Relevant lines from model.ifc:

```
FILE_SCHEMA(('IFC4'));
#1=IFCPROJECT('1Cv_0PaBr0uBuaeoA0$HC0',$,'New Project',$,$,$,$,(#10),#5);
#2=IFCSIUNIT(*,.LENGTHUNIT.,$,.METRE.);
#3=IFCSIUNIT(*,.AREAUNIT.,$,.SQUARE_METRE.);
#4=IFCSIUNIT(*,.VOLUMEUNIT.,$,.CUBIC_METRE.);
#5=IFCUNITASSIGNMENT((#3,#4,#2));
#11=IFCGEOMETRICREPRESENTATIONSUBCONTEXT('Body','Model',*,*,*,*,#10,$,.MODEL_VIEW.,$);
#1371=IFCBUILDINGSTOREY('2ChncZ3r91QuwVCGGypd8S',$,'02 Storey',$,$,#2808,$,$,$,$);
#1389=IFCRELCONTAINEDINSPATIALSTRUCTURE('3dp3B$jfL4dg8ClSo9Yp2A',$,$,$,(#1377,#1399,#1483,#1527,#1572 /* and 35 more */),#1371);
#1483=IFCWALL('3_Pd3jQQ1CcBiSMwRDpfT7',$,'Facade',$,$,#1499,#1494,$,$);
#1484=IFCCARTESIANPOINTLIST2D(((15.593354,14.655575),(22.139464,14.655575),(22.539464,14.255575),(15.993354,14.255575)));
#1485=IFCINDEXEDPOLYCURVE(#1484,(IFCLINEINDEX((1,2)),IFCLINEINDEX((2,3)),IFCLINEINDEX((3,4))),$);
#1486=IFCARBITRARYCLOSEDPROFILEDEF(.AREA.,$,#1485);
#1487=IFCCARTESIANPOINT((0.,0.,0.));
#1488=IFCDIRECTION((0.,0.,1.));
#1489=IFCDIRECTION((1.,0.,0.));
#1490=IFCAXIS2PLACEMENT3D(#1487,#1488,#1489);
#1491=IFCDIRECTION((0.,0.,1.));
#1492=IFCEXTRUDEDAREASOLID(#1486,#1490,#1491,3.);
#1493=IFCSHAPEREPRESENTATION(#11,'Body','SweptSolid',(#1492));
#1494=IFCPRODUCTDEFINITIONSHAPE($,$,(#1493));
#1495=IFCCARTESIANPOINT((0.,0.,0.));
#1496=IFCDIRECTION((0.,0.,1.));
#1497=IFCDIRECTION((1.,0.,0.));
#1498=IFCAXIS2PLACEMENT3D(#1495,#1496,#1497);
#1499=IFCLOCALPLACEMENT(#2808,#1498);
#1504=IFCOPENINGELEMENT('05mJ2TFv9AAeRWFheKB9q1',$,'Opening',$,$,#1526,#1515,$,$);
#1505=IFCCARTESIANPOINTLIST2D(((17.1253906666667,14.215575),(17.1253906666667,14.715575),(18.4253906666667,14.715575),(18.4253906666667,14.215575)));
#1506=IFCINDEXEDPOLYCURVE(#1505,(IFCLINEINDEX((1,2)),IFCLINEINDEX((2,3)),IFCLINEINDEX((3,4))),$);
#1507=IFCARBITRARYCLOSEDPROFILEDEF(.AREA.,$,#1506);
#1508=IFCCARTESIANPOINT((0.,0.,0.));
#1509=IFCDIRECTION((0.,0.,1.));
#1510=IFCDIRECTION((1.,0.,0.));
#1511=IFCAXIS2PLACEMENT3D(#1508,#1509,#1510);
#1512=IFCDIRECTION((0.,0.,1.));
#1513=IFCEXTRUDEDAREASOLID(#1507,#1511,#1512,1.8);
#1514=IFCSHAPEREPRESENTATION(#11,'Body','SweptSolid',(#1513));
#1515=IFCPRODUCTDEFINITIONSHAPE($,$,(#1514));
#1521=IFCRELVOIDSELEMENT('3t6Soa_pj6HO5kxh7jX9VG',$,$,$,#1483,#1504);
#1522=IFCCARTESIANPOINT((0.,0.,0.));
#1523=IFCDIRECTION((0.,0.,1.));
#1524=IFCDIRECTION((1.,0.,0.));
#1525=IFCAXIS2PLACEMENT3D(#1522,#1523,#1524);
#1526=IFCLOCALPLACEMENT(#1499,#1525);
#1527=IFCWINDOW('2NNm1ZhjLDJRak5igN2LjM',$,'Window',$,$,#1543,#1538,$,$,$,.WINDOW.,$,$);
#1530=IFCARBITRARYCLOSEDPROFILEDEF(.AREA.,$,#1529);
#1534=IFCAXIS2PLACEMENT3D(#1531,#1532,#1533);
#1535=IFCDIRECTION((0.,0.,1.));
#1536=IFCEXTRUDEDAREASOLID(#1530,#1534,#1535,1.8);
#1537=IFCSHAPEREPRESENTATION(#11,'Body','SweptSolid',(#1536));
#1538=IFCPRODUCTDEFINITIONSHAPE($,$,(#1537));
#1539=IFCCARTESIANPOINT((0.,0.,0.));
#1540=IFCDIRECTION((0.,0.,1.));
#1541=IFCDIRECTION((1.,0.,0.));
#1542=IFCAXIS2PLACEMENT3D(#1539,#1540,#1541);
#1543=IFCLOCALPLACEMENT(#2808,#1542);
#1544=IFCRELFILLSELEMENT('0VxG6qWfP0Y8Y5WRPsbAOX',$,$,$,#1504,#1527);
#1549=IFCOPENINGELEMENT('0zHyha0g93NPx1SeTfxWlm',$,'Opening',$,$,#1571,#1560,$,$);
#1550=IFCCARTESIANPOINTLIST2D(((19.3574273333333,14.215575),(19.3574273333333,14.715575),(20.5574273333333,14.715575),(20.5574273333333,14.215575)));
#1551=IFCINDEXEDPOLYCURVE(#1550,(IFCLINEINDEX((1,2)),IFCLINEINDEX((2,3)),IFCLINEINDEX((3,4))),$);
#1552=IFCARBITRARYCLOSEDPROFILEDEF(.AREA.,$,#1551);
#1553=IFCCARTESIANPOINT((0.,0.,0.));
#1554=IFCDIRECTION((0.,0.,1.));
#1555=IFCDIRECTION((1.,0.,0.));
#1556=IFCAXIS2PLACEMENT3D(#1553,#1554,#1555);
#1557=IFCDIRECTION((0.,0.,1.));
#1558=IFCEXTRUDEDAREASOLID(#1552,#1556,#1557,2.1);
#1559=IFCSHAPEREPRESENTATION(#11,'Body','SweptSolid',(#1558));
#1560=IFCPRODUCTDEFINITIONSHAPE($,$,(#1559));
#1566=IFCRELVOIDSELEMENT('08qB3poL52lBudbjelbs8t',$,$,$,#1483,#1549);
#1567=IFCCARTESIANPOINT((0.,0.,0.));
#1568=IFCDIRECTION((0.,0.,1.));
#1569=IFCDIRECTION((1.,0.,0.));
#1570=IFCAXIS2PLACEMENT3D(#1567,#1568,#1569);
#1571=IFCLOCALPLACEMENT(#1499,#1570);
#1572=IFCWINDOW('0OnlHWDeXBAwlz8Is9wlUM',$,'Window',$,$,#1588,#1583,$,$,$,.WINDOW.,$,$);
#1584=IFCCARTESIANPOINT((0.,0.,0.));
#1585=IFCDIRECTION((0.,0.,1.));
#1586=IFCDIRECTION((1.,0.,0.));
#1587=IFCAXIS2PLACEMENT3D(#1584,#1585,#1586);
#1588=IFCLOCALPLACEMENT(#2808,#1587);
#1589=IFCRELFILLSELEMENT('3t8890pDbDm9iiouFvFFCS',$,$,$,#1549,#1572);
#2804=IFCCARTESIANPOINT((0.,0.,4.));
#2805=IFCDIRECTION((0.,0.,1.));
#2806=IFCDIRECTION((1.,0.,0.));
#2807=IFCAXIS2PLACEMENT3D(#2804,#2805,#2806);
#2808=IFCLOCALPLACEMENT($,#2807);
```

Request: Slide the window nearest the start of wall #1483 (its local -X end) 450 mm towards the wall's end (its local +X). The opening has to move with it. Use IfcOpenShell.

```python
import ifcopenshell
import ifcopenshell.api.geometry
import ifcopenshell.util.placement
import ifcopenshell.util.unit

model = ifcopenshell.open("model.ifc")
unit_scale = ifcopenshell.util.unit.calculate_unit_scale(model)

window = model.by_guid("2NNm1ZhjLDJRak5igN2LjM")
opening = window.FillsVoids[0].RelatingOpeningElement
wall = opening.VoidsElements[0].RelatingBuildingElement

wall_matrix = ifcopenshell.util.placement.get_local_placement(wall.ObjectPlacement)
shift = wall_matrix[:3, 0] * 0.45 / unit_scale
before = ifcopenshell.util.placement.get_local_placement(window.ObjectPlacement)[:3, 3].copy()

# The window is not placed relative to its opening, so move both.
for product in (opening, window):
    matrix = ifcopenshell.util.placement.get_local_placement(product.ObjectPlacement)
    matrix[:3, 3] += shift
    ifcopenshell.api.geometry.edit_object_placement(model, product=product, matrix=matrix, is_si=False)

after = ifcopenshell.util.placement.get_local_placement(window.ObjectPlacement)[:3, 3]
print("window moved by", (after - before).round(3) + 0.0)

model.write("model_edited.ifc")
```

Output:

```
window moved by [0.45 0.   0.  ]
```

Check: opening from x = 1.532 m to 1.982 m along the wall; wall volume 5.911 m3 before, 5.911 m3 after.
